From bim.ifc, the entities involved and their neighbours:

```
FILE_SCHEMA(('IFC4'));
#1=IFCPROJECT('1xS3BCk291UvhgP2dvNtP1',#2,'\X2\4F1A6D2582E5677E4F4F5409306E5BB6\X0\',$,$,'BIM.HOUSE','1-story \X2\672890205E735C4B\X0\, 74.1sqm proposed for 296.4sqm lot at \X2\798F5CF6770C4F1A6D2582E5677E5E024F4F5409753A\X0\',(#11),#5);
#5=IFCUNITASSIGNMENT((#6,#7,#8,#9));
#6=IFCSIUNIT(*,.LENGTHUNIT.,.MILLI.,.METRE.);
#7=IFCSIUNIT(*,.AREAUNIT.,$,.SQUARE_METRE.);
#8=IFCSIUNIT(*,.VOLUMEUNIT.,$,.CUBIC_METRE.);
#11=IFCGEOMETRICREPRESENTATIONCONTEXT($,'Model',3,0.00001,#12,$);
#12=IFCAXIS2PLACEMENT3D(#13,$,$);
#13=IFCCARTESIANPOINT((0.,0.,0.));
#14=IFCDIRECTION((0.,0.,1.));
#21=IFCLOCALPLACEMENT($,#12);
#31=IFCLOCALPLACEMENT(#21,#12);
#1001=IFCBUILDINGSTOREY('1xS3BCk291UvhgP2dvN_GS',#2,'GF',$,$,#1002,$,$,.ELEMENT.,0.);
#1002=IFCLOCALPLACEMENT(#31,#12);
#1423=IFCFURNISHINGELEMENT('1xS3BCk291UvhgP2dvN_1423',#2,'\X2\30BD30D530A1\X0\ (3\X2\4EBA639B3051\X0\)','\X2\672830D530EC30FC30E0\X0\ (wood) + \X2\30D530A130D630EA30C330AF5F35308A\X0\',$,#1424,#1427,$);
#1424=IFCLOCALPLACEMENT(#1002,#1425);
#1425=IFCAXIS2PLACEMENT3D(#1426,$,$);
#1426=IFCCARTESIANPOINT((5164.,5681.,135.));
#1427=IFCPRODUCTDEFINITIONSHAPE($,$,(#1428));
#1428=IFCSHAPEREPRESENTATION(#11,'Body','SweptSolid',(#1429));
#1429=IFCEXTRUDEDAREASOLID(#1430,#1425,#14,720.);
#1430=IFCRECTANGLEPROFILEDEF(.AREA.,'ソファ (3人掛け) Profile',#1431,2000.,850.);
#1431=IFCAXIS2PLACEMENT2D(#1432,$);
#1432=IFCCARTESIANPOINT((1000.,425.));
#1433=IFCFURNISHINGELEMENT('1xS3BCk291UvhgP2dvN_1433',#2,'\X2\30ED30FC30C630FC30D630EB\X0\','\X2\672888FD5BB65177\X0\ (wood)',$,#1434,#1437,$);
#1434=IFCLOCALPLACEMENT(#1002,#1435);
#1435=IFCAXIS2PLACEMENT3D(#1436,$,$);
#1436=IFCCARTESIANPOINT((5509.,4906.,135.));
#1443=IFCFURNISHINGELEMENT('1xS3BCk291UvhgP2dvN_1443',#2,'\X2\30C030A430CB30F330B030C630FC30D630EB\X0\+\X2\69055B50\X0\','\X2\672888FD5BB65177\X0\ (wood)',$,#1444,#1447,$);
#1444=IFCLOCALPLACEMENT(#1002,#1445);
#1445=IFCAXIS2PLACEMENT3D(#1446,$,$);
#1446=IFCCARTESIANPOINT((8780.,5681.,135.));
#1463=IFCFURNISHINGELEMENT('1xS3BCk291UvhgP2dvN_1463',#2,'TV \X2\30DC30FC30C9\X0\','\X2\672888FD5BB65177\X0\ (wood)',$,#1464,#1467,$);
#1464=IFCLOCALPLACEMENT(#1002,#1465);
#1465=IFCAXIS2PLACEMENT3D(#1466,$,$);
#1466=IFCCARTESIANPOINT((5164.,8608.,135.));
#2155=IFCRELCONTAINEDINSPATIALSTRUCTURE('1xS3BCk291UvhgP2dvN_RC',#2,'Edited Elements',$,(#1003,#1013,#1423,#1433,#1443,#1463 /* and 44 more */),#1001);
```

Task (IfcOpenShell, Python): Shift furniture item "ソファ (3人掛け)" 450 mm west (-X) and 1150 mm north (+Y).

```python
import ifcopenshell
import ifcopenshell.api.geometry
import ifcopenshell.util.placement
import ifcopenshell.util.unit

model = ifcopenshell.open("bim.ifc")
unit_scale = ifcopenshell.util.unit.calculate_unit_scale(model)

item = model.by_guid("1xS3BCk291UvhgP2dvN_1423")
matrix = ifcopenshell.util.placement.get_local_placement(item.ObjectPlacement)
matrix[0, 3] -= 0.45 / unit_scale
matrix[1, 3] += 1.15 / unit_scale
ifcopenshell.api.geometry.edit_object_placement(model, product=item, matrix=matrix, is_si=False)

print(ifcopenshell.util.placement.get_local_placement(item.ObjectPlacement).round(3) + 0.0)

model.write("bim_edited.ifc")
```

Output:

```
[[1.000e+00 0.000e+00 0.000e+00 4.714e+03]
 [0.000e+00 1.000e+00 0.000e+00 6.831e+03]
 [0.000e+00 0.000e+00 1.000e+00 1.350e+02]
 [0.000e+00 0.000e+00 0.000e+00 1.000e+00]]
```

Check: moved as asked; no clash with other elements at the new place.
